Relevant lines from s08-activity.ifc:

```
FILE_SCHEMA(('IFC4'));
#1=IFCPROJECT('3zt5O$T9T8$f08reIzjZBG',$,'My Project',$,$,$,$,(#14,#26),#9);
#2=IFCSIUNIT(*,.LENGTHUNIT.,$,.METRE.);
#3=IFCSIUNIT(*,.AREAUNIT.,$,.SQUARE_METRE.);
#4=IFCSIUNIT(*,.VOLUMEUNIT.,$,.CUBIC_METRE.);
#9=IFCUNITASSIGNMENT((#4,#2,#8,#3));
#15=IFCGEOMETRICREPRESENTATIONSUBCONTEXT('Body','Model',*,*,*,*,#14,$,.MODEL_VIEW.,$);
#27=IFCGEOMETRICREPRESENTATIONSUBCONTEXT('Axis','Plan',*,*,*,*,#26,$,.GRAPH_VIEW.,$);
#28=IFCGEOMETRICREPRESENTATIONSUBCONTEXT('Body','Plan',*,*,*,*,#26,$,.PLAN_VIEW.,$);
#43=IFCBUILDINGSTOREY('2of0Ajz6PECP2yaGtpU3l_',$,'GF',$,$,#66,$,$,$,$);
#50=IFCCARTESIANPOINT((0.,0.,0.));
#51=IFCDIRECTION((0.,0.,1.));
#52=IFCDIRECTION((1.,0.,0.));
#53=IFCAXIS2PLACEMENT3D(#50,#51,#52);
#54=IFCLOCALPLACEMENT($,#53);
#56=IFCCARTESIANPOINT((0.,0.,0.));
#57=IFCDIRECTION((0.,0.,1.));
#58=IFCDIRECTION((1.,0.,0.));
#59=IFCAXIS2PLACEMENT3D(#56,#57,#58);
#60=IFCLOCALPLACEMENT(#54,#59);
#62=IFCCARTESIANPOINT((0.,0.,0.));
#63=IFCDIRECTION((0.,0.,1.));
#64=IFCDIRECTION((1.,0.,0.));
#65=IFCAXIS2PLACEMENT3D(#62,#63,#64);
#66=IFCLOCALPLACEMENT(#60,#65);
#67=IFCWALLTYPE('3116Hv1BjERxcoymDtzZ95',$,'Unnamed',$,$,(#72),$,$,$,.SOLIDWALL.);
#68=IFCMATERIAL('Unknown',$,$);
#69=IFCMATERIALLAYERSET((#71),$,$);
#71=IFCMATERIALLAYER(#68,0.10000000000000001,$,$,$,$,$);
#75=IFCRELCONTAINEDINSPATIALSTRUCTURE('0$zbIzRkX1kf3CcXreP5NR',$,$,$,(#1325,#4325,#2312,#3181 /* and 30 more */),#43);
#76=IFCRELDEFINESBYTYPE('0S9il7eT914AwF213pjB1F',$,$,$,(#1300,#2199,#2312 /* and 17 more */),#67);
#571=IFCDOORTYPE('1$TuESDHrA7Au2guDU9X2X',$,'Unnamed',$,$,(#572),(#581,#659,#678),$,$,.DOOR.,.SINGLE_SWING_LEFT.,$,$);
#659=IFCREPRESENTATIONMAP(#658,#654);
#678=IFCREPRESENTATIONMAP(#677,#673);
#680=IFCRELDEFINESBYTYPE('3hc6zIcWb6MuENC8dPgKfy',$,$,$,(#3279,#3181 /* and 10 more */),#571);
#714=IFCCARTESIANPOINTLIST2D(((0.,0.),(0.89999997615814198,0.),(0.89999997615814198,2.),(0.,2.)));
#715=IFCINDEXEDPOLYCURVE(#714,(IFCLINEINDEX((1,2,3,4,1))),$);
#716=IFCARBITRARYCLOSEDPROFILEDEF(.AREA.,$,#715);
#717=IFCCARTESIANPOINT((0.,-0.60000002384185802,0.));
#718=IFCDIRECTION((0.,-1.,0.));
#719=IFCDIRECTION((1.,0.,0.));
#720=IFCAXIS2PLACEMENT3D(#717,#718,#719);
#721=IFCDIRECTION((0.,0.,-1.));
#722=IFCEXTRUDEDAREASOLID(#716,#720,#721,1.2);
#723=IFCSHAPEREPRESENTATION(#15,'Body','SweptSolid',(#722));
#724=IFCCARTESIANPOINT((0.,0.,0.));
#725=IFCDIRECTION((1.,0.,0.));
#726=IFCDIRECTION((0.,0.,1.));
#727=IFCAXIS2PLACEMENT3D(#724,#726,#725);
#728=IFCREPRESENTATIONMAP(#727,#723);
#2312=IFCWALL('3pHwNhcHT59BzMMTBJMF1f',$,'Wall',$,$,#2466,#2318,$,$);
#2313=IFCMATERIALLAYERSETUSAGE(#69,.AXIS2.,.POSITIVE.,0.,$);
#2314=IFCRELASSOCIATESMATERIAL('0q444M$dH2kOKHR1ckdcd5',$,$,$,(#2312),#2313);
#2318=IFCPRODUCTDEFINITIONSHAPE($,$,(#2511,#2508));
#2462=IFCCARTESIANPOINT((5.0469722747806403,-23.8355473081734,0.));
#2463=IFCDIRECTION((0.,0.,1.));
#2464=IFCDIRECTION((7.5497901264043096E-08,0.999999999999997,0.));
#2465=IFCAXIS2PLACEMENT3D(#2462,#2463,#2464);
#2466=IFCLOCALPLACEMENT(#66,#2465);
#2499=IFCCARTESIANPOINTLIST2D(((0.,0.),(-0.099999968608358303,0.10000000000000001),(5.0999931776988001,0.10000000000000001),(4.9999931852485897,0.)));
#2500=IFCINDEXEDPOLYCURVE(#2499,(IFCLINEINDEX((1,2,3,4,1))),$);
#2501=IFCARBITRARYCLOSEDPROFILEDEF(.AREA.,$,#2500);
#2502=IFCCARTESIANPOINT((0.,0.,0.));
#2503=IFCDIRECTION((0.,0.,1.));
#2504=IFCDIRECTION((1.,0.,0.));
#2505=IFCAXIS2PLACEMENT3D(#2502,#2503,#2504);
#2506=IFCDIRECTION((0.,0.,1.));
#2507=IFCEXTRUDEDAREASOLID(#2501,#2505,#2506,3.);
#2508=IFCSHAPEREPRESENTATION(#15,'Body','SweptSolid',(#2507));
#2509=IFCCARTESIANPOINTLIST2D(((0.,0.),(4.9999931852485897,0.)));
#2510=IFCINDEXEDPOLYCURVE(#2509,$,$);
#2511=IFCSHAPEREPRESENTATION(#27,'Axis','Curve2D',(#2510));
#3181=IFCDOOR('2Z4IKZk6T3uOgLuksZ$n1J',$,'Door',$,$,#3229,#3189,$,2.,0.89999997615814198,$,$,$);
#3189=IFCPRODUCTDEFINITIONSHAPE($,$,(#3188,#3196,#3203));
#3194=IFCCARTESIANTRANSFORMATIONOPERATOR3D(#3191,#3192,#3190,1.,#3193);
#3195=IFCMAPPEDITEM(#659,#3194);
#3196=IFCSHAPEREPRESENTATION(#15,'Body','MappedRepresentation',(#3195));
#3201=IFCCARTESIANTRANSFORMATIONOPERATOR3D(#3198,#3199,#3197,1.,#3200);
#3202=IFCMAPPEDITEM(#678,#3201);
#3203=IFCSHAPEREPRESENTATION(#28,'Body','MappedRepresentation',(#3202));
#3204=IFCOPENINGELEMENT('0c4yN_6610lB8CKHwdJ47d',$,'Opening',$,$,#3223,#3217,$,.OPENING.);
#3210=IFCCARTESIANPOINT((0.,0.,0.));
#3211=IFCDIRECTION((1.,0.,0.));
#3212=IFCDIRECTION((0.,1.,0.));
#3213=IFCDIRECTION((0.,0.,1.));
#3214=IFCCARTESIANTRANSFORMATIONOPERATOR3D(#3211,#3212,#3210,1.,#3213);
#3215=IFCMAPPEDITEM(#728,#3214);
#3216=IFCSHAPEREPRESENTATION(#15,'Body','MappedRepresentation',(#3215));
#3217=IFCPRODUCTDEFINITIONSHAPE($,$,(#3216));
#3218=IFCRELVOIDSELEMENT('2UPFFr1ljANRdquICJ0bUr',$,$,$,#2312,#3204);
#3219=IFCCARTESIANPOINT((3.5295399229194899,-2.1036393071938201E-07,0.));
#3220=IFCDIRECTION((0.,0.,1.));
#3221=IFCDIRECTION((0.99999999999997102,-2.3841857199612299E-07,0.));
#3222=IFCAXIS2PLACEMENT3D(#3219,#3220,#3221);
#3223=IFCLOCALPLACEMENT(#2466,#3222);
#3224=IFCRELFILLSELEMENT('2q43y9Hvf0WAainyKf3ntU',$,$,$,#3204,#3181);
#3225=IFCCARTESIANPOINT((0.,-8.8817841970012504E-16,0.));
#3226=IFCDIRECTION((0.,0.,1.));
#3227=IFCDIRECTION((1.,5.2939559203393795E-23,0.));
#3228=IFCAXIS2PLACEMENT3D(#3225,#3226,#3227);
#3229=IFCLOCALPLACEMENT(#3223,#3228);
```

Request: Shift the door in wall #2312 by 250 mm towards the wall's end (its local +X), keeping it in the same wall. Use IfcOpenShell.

```python
import ifcopenshell
import ifcopenshell.api.geometry
import ifcopenshell.util.placement
import ifcopenshell.util.unit

model = ifcopenshell.open("s08-activity.ifc")
unit_scale = ifcopenshell.util.unit.calculate_unit_scale(model)

door = model.by_id(3181)
opening = door.FillsVoids[0].RelatingOpeningElement
wall = opening.VoidsElements[0].RelatingBuildingElement

wall_matrix = ifcopenshell.util.placement.get_local_placement(wall.ObjectPlacement)
shift = wall_matrix[:3, 0] * 0.25 / unit_scale
before = ifcopenshell.util.placement.get_local_placement(door.ObjectPlacement)[:3, 3].copy()

# The door is placed relative to its opening, so it follows when the opening moves.
matrix = ifcopenshell.util.placement.get_local_placement(opening.ObjectPlacement)
matrix[:3, 3] += shift
ifcopenshell.api.geometry.edit_object_placement(
    model, product=opening, matrix=matrix, is_si=False, should_transform_children=True
)

after = ifcopenshell.util.placement.get_local_placement(door.ObjectPlacement)[:3, 3]
print("door moved by", (after - before).round(3) + 0.0)

model.write("s08-activity-out.ifc")
```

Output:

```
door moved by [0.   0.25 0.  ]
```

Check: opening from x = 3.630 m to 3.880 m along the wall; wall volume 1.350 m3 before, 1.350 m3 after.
